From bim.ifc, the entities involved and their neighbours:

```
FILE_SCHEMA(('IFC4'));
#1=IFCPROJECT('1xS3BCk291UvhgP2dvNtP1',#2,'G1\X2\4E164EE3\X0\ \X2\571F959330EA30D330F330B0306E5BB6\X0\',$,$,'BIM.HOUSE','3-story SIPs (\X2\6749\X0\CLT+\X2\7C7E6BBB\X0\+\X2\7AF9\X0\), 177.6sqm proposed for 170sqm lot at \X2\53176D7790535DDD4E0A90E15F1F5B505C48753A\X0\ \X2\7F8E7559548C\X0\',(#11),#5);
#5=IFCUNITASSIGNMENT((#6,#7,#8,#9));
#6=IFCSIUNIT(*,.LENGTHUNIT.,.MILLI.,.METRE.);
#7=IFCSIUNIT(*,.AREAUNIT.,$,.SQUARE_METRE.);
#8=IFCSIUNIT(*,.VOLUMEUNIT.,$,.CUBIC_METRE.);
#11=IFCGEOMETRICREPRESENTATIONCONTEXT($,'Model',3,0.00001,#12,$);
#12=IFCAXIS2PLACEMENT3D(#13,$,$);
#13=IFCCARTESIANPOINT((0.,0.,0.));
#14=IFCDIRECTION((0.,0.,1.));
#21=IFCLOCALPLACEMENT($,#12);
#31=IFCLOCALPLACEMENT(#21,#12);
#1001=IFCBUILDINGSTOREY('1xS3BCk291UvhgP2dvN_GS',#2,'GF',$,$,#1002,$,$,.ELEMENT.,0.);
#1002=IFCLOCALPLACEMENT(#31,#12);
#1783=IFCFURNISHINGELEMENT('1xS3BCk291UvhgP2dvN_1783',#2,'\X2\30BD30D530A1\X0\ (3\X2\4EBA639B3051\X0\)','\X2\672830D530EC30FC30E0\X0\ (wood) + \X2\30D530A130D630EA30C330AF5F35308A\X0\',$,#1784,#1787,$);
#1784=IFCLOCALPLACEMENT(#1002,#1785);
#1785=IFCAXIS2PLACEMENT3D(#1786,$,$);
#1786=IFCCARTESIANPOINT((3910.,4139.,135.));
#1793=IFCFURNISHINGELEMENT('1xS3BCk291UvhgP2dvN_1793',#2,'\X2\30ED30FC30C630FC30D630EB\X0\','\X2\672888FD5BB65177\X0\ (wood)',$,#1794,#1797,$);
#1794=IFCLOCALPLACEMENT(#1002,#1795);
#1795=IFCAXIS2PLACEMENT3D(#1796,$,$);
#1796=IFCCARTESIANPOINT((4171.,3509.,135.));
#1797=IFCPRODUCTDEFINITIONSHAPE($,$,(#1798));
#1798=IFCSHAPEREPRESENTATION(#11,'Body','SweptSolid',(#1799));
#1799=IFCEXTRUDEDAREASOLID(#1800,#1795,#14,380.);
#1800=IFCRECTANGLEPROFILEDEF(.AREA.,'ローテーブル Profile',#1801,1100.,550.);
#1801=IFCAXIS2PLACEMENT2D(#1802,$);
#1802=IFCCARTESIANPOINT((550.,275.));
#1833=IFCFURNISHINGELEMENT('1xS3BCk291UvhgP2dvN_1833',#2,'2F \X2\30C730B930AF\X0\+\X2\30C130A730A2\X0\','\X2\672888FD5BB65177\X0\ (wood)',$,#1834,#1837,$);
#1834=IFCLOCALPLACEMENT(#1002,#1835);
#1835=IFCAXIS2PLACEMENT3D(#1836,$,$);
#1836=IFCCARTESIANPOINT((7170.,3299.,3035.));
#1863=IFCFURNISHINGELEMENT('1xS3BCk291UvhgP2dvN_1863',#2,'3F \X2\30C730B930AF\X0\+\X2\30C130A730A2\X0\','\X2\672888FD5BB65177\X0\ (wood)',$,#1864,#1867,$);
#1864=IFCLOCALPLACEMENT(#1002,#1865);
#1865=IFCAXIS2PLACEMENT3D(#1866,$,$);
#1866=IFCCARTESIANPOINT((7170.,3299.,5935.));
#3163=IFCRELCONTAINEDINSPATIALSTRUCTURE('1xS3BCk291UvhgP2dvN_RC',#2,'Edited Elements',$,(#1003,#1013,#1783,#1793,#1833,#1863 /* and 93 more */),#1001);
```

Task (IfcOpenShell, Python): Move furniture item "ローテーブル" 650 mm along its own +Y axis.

```python
import ifcopenshell
import ifcopenshell.api.geometry
import ifcopenshell.util.placement
import ifcopenshell.util.unit

model = ifcopenshell.open("bim.ifc")
unit_scale = ifcopenshell.util.unit.calculate_unit_scale(model)

item = model.by_id(1793)
matrix = ifcopenshell.util.placement.get_local_placement(item.ObjectPlacement)
matrix[:3, 3] += matrix[:3, 1] * 0.65 / unit_scale
ifcopenshell.api.geometry.edit_object_placement(model, product=item, matrix=matrix, is_si=False)

print(ifcopenshell.util.placement.get_local_placement(item.ObjectPlacement).round(3) + 0.0)

model.write("bim_rev.ifc")
```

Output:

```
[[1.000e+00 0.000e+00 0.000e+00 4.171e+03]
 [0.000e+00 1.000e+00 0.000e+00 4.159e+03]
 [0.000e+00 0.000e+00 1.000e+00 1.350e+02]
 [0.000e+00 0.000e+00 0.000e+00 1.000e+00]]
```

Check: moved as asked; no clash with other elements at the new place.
